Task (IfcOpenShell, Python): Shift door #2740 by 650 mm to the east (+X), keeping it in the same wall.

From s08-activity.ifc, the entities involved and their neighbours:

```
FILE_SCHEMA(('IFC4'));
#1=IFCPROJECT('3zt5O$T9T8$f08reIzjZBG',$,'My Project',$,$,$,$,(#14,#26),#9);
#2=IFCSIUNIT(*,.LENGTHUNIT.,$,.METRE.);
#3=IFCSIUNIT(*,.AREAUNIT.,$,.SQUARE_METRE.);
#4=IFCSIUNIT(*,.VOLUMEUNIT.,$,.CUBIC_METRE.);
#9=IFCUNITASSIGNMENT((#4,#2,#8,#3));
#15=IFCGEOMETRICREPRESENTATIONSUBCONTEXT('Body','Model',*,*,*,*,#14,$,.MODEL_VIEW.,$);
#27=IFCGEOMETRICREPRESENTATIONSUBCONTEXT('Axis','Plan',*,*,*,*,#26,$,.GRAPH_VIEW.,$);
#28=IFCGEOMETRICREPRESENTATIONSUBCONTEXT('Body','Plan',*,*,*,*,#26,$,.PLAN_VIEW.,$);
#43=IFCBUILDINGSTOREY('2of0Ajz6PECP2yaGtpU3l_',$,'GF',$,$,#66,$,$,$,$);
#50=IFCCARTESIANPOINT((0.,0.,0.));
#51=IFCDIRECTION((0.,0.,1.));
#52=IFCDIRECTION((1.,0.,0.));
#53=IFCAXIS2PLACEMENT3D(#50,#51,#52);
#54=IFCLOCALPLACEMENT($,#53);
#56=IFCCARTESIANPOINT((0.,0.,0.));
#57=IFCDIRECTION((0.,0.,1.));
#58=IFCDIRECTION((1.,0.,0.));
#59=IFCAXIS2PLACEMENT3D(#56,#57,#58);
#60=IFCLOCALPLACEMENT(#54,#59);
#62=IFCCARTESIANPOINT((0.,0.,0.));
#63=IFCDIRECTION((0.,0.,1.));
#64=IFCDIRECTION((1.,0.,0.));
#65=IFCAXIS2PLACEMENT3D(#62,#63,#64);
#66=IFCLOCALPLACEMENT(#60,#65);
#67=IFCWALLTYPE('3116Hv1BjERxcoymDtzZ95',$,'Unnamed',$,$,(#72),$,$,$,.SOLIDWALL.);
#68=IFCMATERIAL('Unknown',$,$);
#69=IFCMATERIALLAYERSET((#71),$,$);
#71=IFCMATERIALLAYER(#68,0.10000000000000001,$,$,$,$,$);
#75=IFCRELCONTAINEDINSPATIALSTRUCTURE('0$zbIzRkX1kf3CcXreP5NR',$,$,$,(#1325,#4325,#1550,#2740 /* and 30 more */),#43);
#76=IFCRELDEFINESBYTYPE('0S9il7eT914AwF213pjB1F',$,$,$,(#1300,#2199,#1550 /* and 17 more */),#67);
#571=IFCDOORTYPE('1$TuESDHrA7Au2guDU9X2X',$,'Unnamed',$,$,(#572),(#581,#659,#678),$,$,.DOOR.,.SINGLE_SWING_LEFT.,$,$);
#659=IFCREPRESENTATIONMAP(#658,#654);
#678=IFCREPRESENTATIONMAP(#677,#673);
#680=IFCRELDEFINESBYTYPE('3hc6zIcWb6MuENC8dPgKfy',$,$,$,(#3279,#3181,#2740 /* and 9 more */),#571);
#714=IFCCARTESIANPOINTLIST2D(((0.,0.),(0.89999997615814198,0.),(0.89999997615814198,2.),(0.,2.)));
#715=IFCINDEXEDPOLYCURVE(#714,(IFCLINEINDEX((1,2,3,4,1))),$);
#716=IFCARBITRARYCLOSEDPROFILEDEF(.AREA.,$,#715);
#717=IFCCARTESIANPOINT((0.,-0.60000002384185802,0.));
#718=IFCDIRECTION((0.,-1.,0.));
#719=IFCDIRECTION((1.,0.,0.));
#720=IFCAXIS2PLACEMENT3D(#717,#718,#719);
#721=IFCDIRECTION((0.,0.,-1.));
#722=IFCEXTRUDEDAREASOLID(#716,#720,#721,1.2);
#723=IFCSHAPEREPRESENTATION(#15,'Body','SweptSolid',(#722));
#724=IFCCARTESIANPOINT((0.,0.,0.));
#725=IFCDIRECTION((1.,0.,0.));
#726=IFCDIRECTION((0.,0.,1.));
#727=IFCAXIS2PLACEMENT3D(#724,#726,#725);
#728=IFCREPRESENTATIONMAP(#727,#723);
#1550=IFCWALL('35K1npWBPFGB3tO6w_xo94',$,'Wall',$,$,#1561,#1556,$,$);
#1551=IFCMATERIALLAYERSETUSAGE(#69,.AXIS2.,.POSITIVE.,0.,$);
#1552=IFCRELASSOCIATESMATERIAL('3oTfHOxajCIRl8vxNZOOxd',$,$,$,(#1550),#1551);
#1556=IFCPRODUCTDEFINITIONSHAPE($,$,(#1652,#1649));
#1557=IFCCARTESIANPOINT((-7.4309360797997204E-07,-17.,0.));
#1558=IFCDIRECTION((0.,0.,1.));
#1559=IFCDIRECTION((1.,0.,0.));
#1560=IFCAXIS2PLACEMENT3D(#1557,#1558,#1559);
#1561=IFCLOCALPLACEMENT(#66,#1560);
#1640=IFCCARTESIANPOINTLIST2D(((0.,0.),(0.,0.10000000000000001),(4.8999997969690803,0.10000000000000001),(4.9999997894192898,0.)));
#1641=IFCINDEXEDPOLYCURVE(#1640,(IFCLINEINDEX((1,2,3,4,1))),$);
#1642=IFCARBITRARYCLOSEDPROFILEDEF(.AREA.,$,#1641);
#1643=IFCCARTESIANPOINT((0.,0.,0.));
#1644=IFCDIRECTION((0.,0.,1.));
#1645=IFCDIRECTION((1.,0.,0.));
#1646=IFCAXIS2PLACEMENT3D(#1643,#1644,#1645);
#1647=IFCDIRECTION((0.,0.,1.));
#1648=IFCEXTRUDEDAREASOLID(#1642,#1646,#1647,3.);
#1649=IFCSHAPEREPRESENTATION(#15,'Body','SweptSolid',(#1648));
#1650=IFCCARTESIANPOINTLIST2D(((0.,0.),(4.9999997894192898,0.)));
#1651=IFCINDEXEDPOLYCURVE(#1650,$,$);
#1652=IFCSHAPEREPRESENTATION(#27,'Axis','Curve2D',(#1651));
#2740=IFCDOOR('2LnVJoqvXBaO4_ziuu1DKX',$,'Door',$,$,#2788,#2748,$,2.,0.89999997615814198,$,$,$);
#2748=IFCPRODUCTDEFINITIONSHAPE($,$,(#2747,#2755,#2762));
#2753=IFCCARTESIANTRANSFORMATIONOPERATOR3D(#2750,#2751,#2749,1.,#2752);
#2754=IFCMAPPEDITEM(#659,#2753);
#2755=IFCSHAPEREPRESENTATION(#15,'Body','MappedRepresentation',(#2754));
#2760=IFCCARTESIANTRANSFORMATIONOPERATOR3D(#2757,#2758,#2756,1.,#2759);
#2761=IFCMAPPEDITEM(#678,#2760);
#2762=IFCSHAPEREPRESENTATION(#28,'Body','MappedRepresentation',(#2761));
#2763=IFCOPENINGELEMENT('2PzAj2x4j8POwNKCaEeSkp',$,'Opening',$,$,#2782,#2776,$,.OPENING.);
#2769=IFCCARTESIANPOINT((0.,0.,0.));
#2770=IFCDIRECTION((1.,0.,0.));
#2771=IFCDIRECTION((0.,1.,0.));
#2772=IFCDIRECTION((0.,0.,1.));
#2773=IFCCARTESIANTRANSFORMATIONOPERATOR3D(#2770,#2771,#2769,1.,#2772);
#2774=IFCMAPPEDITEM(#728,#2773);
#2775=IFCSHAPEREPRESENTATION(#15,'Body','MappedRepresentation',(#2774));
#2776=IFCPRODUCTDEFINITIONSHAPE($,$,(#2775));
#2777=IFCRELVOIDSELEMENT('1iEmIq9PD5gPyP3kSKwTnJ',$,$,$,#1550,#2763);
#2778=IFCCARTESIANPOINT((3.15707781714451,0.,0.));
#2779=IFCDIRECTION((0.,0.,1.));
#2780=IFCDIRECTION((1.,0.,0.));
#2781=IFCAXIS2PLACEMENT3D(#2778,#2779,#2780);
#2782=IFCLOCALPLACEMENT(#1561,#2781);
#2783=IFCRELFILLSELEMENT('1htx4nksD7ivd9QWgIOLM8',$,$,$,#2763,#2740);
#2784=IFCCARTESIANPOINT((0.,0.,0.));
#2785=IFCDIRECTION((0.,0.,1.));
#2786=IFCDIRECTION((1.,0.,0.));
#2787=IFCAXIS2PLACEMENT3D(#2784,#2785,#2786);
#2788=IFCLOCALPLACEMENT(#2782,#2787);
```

```python
import ifcopenshell
import ifcopenshell.api.geometry
import ifcopenshell.util.placement

model = ifcopenshell.open("s08-activity.ifc")

door = model.by_guid("2LnVJoqvXBaO4_ziuu1DKX")
opening = door.FillsVoids[0].RelatingOpeningElement
wall = opening.VoidsElements[0].RelatingBuildingElement

wall_matrix = ifcopenshell.util.placement.get_local_placement(wall.ObjectPlacement)
shift = wall_matrix[:3, 0] * 0.65
before = ifcopenshell.util.placement.get_local_placement(door.ObjectPlacement)[:3, 3].copy()

# The door is placed relative to its opening, so it follows when the opening moves.
matrix = ifcopenshell.util.placement.get_local_placement(opening.ObjectPlacement)
matrix[:3, 3] += shift
ifcopenshell.api.geometry.edit_object_placement(
    model, product=opening, matrix=matrix, is_si=False, should_transform_children=True
)

after = ifcopenshell.util.placement.get_local_placement(door.ObjectPlacement)[:3, 3]
print("door moved by", (after - before).round(3) + 0.0)

model.write("s08-activity_rev.ifc")
```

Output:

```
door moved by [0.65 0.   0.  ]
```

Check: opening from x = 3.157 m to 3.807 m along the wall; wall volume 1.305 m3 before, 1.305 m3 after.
